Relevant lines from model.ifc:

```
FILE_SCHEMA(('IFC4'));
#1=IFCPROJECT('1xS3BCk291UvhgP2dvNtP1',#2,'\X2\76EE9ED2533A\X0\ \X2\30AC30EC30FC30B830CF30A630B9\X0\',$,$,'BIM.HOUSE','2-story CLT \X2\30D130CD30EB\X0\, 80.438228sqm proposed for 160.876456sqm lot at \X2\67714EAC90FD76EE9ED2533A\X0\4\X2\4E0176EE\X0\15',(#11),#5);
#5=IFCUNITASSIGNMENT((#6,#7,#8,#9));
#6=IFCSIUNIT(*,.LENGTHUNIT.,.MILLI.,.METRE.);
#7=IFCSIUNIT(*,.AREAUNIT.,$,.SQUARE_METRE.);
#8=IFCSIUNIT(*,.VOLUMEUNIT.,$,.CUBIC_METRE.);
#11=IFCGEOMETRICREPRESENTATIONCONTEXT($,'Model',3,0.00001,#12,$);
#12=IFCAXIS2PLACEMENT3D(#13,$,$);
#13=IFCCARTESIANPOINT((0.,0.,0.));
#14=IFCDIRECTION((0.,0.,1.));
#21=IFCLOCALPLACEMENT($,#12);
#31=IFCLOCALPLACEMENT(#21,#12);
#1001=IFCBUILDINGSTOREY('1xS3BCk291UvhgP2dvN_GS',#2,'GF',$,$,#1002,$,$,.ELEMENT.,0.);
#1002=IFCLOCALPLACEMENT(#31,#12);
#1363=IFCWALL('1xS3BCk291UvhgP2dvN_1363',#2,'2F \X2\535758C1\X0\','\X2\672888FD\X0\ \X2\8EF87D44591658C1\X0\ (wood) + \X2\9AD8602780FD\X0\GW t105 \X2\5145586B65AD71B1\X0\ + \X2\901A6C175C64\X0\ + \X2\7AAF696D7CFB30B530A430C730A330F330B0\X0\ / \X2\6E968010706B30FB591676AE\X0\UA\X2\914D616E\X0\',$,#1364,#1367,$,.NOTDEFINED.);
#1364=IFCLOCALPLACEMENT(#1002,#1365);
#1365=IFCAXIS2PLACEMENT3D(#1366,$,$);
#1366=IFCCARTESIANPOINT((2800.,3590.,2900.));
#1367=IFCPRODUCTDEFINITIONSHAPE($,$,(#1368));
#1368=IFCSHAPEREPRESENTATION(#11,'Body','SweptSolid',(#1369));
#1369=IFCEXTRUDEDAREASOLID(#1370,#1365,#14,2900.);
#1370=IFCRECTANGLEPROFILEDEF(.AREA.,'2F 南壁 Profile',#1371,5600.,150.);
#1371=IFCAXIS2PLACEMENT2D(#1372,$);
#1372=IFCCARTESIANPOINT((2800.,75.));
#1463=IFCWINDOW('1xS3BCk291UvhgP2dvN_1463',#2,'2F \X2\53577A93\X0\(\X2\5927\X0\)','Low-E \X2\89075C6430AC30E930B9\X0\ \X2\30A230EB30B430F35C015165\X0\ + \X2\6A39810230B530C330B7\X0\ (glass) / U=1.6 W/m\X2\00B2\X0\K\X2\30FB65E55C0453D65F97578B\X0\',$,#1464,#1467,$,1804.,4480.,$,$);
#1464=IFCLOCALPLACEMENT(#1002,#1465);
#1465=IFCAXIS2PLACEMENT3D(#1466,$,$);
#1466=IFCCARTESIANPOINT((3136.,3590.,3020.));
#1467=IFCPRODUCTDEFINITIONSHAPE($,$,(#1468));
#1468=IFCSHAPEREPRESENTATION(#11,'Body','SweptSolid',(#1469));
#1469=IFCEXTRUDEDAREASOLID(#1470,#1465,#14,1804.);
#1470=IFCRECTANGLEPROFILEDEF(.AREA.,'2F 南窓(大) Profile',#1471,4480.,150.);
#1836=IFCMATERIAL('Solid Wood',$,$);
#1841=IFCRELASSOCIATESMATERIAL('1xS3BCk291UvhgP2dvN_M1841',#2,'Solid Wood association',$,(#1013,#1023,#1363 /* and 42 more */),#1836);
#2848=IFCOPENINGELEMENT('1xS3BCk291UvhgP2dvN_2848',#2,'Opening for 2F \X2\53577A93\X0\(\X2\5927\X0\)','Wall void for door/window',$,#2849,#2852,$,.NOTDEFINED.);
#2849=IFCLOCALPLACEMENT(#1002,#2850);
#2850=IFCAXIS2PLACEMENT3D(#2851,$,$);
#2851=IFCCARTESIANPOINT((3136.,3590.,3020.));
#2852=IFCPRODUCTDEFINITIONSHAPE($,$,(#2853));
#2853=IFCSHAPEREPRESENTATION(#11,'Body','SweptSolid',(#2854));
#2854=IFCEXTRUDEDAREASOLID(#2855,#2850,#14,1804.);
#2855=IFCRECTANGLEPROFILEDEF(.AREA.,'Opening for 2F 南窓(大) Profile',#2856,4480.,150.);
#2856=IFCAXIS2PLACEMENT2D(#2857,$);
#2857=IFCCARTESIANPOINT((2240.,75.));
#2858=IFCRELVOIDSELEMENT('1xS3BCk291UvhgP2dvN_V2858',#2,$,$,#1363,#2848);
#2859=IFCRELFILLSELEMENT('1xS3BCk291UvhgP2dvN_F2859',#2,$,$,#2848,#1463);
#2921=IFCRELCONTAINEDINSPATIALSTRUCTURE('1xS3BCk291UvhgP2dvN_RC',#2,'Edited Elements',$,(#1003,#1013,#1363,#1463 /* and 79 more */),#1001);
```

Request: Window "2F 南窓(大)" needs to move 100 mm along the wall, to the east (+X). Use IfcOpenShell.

```python
import ifcopenshell
import ifcopenshell.api.geometry
import ifcopenshell.util.placement

model = ifcopenshell.open("model.ifc")

window = model.by_guid("1xS3BCk291UvhgP2dvN_1463")
opening = window.FillsVoids[0].RelatingOpeningElement
wall = opening.VoidsElements[0].RelatingBuildingElement

wall_matrix = ifcopenshell.util.placement.get_local_placement(wall.ObjectPlacement)
shift = wall_matrix[:3, 0] * 100.0
before = ifcopenshell.util.placement.get_local_placement(window.ObjectPlacement)[:3, 3].copy()

# The window is not placed relative to its opening, so move both.
for product in (opening, window):
    matrix = ifcopenshell.util.placement.get_local_placement(product.ObjectPlacement)
    matrix[:3, 3] += shift
    ifcopenshell.api.geometry.edit_object_placement(model, product=product, matrix=matrix, is_si=False)

after = ifcopenshell.util.placement.get_local_placement(window.ObjectPlacement)[:3, 3]
print("window moved by", (after - before).round(3) + 0.0)

model.write("model_updated.ifc")
```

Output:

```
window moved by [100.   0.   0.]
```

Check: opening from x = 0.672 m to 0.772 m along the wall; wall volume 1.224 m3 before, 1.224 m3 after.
